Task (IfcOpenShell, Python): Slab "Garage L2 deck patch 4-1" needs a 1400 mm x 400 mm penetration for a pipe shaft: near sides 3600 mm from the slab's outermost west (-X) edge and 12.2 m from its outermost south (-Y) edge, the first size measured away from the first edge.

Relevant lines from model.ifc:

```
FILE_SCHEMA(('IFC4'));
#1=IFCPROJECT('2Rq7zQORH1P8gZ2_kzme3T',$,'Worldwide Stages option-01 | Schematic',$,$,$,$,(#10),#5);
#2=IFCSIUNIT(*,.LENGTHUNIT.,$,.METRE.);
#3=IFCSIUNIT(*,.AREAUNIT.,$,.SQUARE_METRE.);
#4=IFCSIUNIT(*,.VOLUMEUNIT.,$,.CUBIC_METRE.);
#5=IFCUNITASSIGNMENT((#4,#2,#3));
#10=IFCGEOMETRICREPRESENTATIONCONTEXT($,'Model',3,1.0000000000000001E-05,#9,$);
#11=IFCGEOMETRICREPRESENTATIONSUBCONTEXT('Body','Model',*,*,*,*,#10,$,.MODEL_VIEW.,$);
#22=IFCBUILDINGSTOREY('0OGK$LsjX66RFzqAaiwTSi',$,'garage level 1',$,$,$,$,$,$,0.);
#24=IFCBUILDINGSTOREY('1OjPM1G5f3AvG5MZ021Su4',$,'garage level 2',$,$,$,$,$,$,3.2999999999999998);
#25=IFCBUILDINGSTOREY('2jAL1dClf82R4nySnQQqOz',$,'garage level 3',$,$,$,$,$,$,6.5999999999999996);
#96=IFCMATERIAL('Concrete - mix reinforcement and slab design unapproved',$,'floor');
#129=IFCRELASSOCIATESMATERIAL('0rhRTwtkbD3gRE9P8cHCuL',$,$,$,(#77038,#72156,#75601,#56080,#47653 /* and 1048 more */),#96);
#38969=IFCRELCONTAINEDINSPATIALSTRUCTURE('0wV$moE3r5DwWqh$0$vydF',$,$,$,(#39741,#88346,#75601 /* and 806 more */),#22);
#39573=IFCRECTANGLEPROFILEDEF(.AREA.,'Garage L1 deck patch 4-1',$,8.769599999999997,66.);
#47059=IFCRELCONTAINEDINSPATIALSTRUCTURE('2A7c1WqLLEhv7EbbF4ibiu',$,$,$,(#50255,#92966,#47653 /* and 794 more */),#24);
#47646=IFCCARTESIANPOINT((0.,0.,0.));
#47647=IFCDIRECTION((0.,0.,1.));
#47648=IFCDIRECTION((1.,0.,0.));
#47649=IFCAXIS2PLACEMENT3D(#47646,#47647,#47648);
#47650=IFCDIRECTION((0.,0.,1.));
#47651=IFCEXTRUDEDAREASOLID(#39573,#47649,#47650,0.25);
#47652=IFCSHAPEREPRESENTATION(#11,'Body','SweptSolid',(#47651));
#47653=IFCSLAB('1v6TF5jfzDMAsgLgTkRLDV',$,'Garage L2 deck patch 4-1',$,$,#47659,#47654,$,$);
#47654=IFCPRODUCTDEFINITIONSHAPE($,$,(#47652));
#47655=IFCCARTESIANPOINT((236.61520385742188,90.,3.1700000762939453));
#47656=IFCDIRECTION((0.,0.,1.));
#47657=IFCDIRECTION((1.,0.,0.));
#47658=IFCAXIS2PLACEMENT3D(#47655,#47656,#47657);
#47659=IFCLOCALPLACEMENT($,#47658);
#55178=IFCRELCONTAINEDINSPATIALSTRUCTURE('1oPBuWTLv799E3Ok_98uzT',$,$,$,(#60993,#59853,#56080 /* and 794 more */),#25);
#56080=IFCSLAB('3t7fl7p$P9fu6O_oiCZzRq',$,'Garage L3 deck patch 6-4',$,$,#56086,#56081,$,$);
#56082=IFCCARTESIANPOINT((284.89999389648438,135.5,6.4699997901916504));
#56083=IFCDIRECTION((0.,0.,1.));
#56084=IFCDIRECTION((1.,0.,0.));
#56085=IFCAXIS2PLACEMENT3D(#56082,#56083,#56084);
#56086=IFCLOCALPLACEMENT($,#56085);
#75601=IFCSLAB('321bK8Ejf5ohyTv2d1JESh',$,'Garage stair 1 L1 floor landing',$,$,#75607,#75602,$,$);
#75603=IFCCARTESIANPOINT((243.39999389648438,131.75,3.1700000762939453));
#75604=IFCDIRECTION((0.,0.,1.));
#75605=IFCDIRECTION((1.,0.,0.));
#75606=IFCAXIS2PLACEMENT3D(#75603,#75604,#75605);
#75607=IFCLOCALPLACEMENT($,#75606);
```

```python
import numpy as np
import ifcopenshell
import ifcopenshell.api.feature
import ifcopenshell.api.geometry
import ifcopenshell.api.root
import ifcopenshell.geom
import ifcopenshell.util.placement
import ifcopenshell.util.representation
import ifcopenshell.util.shape
import ifcopenshell.util.unit

model = ifcopenshell.open("model.ifc")
unit_scale = ifcopenshell.util.unit.calculate_unit_scale(model)
settings = ifcopenshell.geom.settings()


def volume(element):
    """Net volume in cubic metres, openings subtracted."""
    shape = ifcopenshell.geom.create_shape(settings, element)
    return ifcopenshell.util.shape.get_volume(shape.geometry)


slab = model.by_id(47653)
before = volume(slab)

# Extent in the slab's own axes, in metres. The edges named are its -X and -Y sides.
slab_shape = ifcopenshell.geom.create_shape(settings, slab)
vertices = ifcopenshell.util.shape.get_vertices(slab_shape.geometry)
x_min, y_min, bottom = vertices.min(axis=0)
top = vertices[:, 2].max()

opening = ifcopenshell.api.root.create_entity(model, ifc_class="IfcOpeningElement", name="Pipe shaft opening", predefined_type="OPENING")
context = ifcopenshell.util.representation.get_context(model, "Model", "Body", "MODEL_VIEW")
width, depth = 1.4, 0.4
outline = [(0.0, 0.0), (width, 0.0), (width, depth), (0.0, depth), (0.0, 0.0)]
# Overshoot both faces by 50 mm so the cut is clean.
shape = ifcopenshell.api.geometry.add_slab_representation(
    model, context=context, depth=top - bottom + 0.1, polyline=outline
)
ifcopenshell.api.geometry.assign_representation(model, product=opening, representation=shape)

matrix = ifcopenshell.util.placement.get_local_placement(slab.ObjectPlacement)
matrix[:, 3] = matrix @ np.append(np.array([x_min + 3.6, y_min + 12.2, bottom - 0.05]) / unit_scale, 1.0)
ifcopenshell.api.geometry.edit_object_placement(model, product=opening, matrix=matrix, is_si=False)
ifcopenshell.api.feature.add_feature(model, feature=opening, element=slab)

after = volume(slab)

print(f"slab volume {before:.3f} -> {after:.3f} m3")

model.write("model_updated.ifc")
```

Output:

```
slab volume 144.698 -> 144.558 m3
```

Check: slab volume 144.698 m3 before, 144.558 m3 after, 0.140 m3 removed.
